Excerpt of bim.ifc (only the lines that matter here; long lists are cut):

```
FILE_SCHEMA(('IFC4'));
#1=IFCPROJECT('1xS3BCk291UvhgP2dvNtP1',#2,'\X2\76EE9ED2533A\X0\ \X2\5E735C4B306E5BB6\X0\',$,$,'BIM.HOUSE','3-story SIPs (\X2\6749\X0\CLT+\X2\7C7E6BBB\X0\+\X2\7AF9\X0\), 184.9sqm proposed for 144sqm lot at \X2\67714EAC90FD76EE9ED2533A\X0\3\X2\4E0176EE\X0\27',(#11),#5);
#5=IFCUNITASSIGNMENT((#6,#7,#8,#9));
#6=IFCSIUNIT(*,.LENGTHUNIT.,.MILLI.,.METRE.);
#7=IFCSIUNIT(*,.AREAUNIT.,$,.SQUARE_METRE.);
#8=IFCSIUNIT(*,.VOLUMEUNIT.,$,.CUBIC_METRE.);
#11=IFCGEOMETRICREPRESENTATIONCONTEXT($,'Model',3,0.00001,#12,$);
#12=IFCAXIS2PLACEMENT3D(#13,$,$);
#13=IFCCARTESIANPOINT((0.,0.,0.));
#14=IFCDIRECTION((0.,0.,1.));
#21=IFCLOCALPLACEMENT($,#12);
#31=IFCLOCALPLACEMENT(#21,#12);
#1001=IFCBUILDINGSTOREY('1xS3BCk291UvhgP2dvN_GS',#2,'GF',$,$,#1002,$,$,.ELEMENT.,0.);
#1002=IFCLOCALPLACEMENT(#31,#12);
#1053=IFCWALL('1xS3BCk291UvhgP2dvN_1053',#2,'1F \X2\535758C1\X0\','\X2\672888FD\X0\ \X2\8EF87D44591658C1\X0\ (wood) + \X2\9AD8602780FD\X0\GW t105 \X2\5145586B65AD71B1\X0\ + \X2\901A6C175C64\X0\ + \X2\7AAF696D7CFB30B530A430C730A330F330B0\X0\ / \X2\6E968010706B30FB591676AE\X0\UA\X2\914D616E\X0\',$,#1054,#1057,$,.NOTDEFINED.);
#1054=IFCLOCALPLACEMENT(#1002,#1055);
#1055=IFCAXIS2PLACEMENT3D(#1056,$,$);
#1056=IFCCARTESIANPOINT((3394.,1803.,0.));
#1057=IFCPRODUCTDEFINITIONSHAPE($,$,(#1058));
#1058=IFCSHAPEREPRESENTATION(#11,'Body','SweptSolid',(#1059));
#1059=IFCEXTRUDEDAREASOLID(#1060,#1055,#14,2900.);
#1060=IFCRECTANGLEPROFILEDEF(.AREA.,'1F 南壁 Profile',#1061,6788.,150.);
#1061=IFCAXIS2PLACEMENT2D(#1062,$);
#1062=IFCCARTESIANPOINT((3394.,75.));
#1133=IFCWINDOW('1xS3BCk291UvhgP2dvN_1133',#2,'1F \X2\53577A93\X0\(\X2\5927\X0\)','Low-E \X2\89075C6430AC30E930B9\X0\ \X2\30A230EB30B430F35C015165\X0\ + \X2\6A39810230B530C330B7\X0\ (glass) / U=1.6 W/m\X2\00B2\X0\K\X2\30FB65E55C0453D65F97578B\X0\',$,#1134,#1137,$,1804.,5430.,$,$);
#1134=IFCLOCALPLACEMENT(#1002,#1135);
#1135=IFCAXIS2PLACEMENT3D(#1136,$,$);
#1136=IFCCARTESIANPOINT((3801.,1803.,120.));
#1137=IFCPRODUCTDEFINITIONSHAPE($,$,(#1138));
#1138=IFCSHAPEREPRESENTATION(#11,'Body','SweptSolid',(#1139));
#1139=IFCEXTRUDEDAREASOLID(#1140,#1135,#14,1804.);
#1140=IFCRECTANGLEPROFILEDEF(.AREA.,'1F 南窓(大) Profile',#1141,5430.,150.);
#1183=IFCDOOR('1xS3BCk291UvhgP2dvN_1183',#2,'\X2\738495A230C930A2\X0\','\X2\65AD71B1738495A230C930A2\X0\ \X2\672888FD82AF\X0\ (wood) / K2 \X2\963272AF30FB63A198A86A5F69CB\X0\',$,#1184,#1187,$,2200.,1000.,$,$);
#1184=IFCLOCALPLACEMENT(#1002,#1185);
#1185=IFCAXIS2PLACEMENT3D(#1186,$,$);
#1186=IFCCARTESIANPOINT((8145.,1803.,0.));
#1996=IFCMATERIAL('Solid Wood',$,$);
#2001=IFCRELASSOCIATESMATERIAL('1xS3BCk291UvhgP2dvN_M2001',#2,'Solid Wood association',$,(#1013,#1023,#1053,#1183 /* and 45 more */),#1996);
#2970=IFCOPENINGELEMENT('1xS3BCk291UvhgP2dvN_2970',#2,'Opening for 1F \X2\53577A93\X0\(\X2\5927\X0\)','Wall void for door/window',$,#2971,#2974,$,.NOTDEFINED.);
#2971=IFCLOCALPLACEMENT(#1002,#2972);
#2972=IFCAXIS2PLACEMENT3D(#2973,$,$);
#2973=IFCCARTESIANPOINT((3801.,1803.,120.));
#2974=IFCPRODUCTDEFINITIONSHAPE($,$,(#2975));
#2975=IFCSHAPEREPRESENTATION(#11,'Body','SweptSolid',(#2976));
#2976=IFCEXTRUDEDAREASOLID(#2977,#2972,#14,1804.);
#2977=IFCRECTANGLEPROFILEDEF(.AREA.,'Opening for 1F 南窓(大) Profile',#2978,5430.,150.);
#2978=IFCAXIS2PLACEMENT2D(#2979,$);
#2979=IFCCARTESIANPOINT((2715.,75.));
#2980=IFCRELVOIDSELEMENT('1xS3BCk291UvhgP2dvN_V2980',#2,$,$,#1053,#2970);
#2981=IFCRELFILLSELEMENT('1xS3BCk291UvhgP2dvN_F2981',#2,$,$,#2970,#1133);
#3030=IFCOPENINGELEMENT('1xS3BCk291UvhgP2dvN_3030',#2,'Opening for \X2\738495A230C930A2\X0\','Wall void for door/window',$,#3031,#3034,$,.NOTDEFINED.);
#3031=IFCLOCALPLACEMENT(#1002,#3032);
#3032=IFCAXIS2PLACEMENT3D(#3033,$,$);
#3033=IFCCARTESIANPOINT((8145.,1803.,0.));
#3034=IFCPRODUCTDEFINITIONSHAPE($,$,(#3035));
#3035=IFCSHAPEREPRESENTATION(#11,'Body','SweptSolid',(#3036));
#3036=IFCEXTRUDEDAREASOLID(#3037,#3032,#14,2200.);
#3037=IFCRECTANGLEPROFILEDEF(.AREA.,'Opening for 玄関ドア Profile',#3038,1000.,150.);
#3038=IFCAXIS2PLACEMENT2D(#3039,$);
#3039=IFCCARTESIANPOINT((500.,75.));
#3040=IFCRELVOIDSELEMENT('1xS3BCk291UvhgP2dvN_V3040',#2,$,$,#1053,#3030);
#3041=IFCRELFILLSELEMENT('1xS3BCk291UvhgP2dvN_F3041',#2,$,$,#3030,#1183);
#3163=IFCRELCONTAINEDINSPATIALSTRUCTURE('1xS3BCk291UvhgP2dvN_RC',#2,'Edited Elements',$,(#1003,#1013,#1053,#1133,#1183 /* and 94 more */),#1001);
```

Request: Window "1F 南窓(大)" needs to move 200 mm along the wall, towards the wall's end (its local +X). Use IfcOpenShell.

```python
import ifcopenshell
import ifcopenshell.api.geometry
import ifcopenshell.util.placement

model = ifcopenshell.open("bim.ifc")

window = model.by_guid("1xS3BCk291UvhgP2dvN_1133")
opening = window.FillsVoids[0].RelatingOpeningElement
wall = opening.VoidsElements[0].RelatingBuildingElement

wall_matrix = ifcopenshell.util.placement.get_local_placement(wall.ObjectPlacement)
shift = wall_matrix[:3, 0] * 200.0
before = ifcopenshell.util.placement.get_local_placement(window.ObjectPlacement)[:3, 3].copy()

# The window is not placed relative to its opening, so move both.
for product in (opening, window):
    matrix = ifcopenshell.util.placement.get_local_placement(product.ObjectPlacement)
    matrix[:3, 3] += shift
    ifcopenshell.api.geometry.edit_object_placement(model, product=product, matrix=matrix, is_si=False)

after = ifcopenshell.util.placement.get_local_placement(window.ObjectPlacement)[:3, 3]
print("window moved by", (after - before).round(3) + 0.0)

model.write("bim-out.ifc")
```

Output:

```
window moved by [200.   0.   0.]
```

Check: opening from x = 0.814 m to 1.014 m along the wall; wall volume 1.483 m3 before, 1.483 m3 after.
